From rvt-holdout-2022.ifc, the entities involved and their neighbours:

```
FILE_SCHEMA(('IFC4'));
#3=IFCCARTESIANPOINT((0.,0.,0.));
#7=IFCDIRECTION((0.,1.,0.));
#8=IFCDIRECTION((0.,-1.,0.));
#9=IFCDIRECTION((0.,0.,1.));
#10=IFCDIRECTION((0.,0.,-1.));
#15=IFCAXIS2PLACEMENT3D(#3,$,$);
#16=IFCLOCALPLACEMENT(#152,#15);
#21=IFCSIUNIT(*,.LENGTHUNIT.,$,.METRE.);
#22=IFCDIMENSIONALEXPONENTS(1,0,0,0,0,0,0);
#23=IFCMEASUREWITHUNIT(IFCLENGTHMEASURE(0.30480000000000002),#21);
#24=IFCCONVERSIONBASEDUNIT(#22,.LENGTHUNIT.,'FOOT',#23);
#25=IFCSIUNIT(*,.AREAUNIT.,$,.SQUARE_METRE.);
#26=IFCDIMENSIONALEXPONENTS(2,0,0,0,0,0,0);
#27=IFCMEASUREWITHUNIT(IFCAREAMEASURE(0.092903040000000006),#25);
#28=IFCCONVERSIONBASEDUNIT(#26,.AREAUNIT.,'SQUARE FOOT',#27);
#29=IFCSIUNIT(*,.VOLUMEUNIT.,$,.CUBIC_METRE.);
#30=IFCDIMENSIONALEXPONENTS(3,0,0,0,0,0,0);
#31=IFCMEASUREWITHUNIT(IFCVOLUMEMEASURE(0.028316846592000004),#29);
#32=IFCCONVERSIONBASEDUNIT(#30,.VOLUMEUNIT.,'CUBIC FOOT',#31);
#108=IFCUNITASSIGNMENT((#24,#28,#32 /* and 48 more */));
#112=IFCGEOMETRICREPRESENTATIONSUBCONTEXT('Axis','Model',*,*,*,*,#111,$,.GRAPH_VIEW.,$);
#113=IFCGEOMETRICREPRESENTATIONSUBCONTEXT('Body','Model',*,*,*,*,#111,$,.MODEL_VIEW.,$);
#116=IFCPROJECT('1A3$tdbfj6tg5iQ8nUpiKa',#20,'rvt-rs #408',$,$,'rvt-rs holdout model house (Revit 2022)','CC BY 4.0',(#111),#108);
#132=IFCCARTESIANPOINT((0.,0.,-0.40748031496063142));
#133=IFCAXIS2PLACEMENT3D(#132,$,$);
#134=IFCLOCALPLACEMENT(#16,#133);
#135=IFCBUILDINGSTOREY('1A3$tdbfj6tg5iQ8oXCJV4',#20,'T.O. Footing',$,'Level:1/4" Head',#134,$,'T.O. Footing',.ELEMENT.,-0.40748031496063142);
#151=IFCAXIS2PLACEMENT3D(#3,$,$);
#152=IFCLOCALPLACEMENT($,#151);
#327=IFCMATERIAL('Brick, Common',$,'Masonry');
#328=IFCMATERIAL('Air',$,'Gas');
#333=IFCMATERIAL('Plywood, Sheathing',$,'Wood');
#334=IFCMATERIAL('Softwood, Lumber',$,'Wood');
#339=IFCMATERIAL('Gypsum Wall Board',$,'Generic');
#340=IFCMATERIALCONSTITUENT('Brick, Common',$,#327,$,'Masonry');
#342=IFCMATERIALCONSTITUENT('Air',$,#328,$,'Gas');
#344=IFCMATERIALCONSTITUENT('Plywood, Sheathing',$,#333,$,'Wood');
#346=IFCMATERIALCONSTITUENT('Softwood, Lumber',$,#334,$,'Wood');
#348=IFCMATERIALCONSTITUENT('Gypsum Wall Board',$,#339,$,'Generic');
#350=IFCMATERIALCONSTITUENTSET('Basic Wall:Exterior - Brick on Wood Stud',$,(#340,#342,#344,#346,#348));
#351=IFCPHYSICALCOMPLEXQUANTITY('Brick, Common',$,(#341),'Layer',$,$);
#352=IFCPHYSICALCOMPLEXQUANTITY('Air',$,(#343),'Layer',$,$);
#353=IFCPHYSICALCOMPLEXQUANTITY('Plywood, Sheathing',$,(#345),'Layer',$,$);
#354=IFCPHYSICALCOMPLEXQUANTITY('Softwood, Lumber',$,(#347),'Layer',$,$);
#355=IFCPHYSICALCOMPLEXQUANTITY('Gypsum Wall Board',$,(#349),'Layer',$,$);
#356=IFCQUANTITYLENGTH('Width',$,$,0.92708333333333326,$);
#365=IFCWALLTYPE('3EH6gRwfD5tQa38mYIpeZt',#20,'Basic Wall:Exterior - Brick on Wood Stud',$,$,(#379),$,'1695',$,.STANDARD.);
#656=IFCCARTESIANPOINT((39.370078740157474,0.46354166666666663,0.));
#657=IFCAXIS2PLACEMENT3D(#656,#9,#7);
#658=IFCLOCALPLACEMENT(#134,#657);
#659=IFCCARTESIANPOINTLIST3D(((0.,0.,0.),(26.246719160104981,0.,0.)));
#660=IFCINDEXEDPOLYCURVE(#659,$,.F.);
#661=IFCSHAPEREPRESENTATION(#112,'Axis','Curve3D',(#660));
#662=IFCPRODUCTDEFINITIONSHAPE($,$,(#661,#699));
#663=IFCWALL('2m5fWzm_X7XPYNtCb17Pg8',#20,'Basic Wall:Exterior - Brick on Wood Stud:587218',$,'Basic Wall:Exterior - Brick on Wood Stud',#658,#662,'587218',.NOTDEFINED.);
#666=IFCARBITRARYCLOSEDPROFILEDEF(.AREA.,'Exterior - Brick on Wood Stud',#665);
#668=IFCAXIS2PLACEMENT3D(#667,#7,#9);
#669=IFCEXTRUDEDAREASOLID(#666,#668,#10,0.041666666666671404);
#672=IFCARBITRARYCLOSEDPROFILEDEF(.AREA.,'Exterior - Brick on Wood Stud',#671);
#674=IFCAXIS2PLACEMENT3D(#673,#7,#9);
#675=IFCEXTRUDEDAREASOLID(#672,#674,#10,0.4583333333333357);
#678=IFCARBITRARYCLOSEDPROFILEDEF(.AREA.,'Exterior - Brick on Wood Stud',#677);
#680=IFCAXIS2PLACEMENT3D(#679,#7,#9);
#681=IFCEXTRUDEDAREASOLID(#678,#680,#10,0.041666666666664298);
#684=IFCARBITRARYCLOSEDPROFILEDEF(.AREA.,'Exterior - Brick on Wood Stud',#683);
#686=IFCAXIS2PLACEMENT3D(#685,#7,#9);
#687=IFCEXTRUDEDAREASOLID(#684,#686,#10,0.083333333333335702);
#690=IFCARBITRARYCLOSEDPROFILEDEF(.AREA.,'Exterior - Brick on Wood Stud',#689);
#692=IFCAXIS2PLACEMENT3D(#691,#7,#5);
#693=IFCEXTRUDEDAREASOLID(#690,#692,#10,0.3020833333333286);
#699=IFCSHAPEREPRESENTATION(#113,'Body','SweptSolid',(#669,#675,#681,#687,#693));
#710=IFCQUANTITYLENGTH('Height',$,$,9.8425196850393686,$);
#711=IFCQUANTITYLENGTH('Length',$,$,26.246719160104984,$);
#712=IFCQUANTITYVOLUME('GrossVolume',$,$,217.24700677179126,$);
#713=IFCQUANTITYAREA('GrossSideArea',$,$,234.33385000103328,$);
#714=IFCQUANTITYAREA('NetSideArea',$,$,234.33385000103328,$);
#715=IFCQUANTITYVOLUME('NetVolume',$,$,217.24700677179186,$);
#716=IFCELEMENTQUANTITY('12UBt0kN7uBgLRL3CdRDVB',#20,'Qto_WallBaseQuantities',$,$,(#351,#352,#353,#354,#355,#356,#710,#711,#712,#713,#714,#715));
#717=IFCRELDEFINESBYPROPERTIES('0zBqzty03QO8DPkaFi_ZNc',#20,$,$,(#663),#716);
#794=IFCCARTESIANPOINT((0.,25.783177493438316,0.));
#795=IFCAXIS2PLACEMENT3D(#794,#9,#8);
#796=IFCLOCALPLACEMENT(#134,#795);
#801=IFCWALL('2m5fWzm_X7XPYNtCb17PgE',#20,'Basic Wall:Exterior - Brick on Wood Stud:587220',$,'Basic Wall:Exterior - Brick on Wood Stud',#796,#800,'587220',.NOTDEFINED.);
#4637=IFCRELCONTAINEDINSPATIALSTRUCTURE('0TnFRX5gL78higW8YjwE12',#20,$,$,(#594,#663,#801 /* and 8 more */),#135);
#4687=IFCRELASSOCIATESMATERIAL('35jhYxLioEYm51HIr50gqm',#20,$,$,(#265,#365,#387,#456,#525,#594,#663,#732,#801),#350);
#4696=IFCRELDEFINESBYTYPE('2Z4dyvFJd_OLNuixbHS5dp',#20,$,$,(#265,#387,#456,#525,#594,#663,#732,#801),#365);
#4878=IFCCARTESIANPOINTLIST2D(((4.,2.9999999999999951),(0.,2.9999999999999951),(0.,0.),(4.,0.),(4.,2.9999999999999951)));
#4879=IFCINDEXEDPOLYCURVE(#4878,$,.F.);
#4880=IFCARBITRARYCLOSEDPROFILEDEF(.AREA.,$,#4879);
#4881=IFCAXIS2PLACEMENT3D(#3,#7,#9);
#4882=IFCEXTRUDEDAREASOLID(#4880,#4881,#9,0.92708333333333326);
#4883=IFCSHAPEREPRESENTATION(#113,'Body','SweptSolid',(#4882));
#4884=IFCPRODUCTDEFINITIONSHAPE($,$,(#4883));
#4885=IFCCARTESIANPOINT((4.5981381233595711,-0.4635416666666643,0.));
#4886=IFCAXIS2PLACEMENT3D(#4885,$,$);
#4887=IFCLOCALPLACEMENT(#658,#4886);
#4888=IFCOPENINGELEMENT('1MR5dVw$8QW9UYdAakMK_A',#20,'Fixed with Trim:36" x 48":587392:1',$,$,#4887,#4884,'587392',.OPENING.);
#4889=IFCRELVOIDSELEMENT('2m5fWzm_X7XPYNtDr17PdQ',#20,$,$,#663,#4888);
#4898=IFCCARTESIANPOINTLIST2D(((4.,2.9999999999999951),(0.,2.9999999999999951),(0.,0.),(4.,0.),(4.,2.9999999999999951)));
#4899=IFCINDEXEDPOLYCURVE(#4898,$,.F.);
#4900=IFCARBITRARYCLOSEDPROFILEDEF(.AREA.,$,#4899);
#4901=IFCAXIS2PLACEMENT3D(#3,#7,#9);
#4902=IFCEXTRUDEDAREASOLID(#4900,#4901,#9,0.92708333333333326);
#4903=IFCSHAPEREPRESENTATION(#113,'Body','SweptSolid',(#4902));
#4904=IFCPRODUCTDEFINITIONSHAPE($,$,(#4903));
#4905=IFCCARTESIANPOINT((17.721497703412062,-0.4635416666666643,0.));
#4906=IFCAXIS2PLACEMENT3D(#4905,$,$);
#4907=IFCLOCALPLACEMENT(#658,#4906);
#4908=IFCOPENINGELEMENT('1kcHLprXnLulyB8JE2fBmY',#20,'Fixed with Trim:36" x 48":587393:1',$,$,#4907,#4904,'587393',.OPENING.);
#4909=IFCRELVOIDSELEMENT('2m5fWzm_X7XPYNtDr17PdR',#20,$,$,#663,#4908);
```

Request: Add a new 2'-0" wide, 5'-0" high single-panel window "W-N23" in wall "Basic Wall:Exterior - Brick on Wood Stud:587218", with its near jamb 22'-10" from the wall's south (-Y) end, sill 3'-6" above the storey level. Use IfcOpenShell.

```python
import numpy as np
import ifcopenshell
import ifcopenshell.api.feature
import ifcopenshell.api.geometry
import ifcopenshell.api.pset
import ifcopenshell.api.root
import ifcopenshell.api.spatial
import ifcopenshell.geom
import ifcopenshell.util.element
import ifcopenshell.util.placement
import ifcopenshell.util.representation
import ifcopenshell.util.shape
import ifcopenshell.util.unit

model = ifcopenshell.open("rvt-holdout-2022.ifc")
unit_scale = ifcopenshell.util.unit.calculate_unit_scale(model)
area_scale = ifcopenshell.util.unit.calculate_unit_scale(model, "AREAUNIT")
volume_scale = ifcopenshell.util.unit.calculate_unit_scale(model, "VOLUMEUNIT")
settings = ifcopenshell.geom.settings()


def volume(element):
    """Net volume in cubic metres, openings subtracted."""
    shape = ifcopenshell.geom.create_shape(settings, element)
    return ifcopenshell.util.shape.get_volume(shape.geometry)


wall = model.by_id(663)
storey = ifcopenshell.util.element.get_container(wall, ifc_class="IfcBuildingStorey")
context = ifcopenshell.util.representation.get_context(model, "Model", "Body", "MODEL_VIEW")
before = volume(wall)

width, height, from_end, sill = 0.6096, 1.524, 6.9596, 1.0668  # metres

# The wall runs along its own X axis, and the end named is its -X end.
wall_shape = ifcopenshell.geom.create_shape(settings, wall)
x, y, z = ifcopenshell.util.shape.get_vertices(wall_shape.geometry).T
start = x.min() + from_end
face, thickness = float(y.min()), float(y.max() - y.min())
wall_matrix = ifcopenshell.util.placement.get_local_placement(wall.ObjectPlacement)
level = ifcopenshell.util.placement.get_local_placement(storey.ObjectPlacement)[2, 3]


def in_wall(x, y):
    """Placement at x, y metres in the wall's axes, at sill height."""
    matrix = wall_matrix.copy()
    matrix[:, 3] = wall_matrix @ np.array([x / unit_scale, y / unit_scale, 0.0, 1.0])
    matrix[2, 3] = level + sill / unit_scale
    return matrix


# Opening: a box that overshoots both wall faces by 50 mm.
opening = ifcopenshell.api.root.create_entity(model, ifc_class="IfcOpeningElement", predefined_type="OPENING")
box = ifcopenshell.api.geometry.add_wall_representation(
    model, context=context, length=width, height=height, thickness=thickness + 0.1
)
ifcopenshell.api.geometry.assign_representation(model, product=opening, representation=box)
ifcopenshell.api.geometry.edit_object_placement(model, product=opening, matrix=in_wall(start, face - 0.05), is_si=False)
ifcopenshell.api.feature.add_feature(model, feature=opening, element=wall)

window = ifcopenshell.api.root.create_entity(model, ifc_class="IfcWindow", name="W-N23", predefined_type="WINDOW")
window.OverallWidth, window.OverallHeight = width / unit_scale, height / unit_scale
window.PartitioningType = "SINGLE_PANEL"
body = ifcopenshell.api.geometry.add_window_representation(
    model,
    context=context,
    overall_width=window.OverallWidth,
    overall_height=window.OverallHeight,
    partition_type="SINGLE_PANEL",
)
ifcopenshell.api.geometry.assign_representation(model, product=window, representation=body)
ifcopenshell.api.spatial.assign_container(model, products=[window], relating_structure=storey)
ifcopenshell.api.feature.add_filling(model, opening=opening, element=window)

# Centre the window in the wall's thickness.
ifcopenshell.api.geometry.edit_object_placement(model, product=window, matrix=in_wall(start, face), is_si=False)
window_shape = ifcopenshell.geom.create_shape(settings, window)
depth = ifcopenshell.util.shape.get_vertices(window_shape.geometry)[:, 1]
offset = face + thickness / 2 - (depth.min() + depth.max()) / 2
ifcopenshell.api.geometry.edit_object_placement(model, product=window, matrix=in_wall(start, offset), is_si=False)

after = volume(wall)

# Update the wall's stored quantities.
qto = model.by_id(ifcopenshell.util.element.get_pset(wall, "Qto_WallBaseQuantities", should_inherit=False)["id"])
ifcopenshell.api.pset.edit_qto(model, qto=qto, properties={
    "NetSideArea": after / thickness / area_scale,
    "NetVolume": after / volume_scale,
})

print(f"wall volume {before:.3f} -> {after:.3f} m3")

model.write("rvt-holdout-2022_updated.ifc")
```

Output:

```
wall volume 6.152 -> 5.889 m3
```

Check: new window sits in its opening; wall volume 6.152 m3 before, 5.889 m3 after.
